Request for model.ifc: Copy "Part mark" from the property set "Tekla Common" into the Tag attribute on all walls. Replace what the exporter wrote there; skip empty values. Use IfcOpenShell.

First a look at what the model holds.

```python
import ifcopenshell
import ifcopenshell.util.element

model = ifcopenshell.open("model.ifc")
print(model.schema)
walls = model.by_type("IfcWall")
print(len(walls), "walls")
for e in walls[:8]:
    source = ifcopenshell.util.element.get_pset(e, "Tekla Common", "Part mark")
    target = e.Tag
    print(e.id(), repr(source), repr(target), sep=" | ")
```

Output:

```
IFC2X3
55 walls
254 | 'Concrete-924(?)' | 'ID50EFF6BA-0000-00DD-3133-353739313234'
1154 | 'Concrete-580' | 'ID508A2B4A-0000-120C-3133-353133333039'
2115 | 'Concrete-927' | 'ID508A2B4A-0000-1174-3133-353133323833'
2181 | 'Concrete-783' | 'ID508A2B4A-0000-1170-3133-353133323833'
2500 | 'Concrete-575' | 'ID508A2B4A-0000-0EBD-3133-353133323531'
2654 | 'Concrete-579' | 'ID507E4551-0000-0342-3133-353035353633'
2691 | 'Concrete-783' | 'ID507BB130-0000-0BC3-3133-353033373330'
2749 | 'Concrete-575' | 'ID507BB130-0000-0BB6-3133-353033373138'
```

```python
import ifcopenshell
import ifcopenshell.util.element

model = ifcopenshell.open("model.ifc")

count = 0
for e in model.by_type("IfcWall"):
    value = ifcopenshell.util.element.get_pset(e, "Tekla Common", "Part mark")
    current = e.Tag
    if not value or not value.strip() or current == value:
        continue
    e.Tag = value
    count += 1

print(count, "walls updated")

model.write("model_v2.ifc")
```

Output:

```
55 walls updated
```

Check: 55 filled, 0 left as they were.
